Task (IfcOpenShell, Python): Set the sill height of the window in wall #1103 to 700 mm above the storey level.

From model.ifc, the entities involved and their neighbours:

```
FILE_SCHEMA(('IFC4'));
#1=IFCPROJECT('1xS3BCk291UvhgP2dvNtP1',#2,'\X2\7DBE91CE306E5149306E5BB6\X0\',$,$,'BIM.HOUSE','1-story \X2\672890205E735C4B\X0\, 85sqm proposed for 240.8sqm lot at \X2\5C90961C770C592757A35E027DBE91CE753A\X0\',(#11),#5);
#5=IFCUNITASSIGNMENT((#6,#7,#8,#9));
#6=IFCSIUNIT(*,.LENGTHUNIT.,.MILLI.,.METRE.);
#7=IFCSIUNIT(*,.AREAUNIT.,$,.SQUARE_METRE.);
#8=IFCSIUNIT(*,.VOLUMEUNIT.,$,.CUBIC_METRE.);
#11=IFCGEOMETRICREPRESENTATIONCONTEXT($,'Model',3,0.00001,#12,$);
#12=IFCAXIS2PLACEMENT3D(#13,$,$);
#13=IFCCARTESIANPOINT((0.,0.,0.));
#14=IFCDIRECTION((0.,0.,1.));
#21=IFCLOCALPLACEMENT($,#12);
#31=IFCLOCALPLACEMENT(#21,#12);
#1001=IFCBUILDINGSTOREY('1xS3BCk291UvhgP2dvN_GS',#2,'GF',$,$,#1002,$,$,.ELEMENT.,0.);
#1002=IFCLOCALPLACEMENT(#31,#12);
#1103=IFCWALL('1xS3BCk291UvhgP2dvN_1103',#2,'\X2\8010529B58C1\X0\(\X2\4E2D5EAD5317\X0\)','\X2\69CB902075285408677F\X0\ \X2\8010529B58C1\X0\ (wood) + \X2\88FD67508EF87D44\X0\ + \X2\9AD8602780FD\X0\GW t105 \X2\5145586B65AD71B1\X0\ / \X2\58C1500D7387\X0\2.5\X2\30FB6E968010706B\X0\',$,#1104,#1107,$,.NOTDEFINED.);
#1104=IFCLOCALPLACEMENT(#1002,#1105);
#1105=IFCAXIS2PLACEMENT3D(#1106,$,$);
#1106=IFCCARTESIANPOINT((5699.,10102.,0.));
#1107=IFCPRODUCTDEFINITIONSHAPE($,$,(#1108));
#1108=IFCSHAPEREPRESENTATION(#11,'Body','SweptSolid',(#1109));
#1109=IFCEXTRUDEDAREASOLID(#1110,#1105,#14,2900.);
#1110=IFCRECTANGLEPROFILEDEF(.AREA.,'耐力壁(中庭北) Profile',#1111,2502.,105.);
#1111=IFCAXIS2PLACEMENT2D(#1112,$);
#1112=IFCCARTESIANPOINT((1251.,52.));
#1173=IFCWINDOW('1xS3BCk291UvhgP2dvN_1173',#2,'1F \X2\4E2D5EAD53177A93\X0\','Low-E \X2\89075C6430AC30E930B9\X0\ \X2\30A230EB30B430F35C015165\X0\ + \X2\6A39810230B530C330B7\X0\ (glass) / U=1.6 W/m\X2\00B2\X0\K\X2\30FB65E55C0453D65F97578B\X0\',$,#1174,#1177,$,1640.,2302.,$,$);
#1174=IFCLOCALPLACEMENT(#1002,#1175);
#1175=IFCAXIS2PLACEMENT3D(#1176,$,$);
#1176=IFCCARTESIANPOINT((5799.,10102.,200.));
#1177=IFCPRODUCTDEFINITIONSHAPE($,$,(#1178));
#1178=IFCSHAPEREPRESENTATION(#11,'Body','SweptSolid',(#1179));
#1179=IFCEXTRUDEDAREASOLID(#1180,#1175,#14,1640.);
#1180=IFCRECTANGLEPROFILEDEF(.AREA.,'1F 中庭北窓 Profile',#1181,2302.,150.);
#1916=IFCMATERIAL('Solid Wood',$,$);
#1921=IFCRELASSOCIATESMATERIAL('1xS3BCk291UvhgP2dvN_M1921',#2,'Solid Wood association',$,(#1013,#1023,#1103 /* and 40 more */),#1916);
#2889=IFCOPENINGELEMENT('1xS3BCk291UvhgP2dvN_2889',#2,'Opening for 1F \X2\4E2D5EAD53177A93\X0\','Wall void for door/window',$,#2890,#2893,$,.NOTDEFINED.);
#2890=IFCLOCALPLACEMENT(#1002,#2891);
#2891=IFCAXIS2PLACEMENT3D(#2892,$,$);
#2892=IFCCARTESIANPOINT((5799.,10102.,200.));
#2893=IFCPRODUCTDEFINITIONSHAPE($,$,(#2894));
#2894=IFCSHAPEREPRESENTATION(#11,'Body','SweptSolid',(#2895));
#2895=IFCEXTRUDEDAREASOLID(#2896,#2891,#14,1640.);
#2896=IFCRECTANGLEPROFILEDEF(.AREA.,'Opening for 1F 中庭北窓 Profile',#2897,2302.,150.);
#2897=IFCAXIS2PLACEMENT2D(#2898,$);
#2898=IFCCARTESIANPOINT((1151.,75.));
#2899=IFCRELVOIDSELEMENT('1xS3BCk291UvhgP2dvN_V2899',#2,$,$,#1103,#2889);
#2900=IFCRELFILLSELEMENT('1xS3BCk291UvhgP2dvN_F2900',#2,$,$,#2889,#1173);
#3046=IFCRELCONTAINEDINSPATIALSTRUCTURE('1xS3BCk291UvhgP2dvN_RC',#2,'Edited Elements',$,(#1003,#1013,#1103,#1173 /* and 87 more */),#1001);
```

```python
import numpy as np
import ifcopenshell
import ifcopenshell.api.geometry
import ifcopenshell.geom
import ifcopenshell.util.element
import ifcopenshell.util.placement
import ifcopenshell.util.shape
import ifcopenshell.util.unit

model = ifcopenshell.open("model.ifc")
unit_scale = ifcopenshell.util.unit.calculate_unit_scale(model)

window = model.by_id(1173)
opening = window.FillsVoids[0].RelatingOpeningElement
storey = ifcopenshell.util.element.get_container(window, ifc_class="IfcBuildingStorey")
level = ifcopenshell.util.placement.get_local_placement(storey.ObjectPlacement)[2, 3]

# The opening's origin need not be at the sill, so measure its lowest point.
shape = ifcopenshell.geom.create_shape(ifcopenshell.geom.settings(), opening)
bottom = ifcopenshell.util.shape.get_shape_bottom_elevation(shape, shape.geometry) / unit_scale
dz = level + 700.0 - bottom

shift = np.array([0.0, 0.0, dz])
# The window is not placed relative to its opening, so move both.
for product in (opening, window):
    matrix = ifcopenshell.util.placement.get_local_placement(product.ObjectPlacement)
    matrix[:3, 3] += shift
    ifcopenshell.api.geometry.edit_object_placement(model, product=product, matrix=matrix, is_si=False)

print(f"moved by {dz * unit_scale:+.3f} m")

model.write("model_edited.ifc")
```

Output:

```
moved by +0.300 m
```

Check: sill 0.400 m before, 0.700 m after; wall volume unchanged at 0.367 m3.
